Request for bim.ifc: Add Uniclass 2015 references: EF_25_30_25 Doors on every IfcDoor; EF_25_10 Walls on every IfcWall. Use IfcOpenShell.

First a look at what the model holds.

```python
import ifcopenshell

model = ifcopenshell.open("bim.ifc")
print(model.schema)
print("classifications:", [c.Name for c in model.by_type("IfcClassification")])
for ifc_class in ("IfcDoor", "IfcRoof", "IfcStair", "IfcWall", "IfcWindow"):
    print(ifc_class, len(model.by_type(ifc_class)))
```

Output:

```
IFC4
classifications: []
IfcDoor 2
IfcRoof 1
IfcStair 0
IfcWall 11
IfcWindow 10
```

```python
import ifcopenshell
import ifcopenshell.api.classification

model = ifcopenshell.open("bim.ifc")

system = ifcopenshell.api.classification.add_classification(model, classification="Uniclass 2015")

codes = {
    "IfcDoor": ("EF_25_30_25", "Doors"),
    "IfcWall": ("EF_25_10", "Walls"),
}
for ifc_class, (code, name) in codes.items():
    products = model.by_type(ifc_class)
    ifcopenshell.api.classification.add_reference(
        model, products=products, classification=system, identification=code, name=name
    )
    print(code, len(products))

model.write("bim-out.ifc")
```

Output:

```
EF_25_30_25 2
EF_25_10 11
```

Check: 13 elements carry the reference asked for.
